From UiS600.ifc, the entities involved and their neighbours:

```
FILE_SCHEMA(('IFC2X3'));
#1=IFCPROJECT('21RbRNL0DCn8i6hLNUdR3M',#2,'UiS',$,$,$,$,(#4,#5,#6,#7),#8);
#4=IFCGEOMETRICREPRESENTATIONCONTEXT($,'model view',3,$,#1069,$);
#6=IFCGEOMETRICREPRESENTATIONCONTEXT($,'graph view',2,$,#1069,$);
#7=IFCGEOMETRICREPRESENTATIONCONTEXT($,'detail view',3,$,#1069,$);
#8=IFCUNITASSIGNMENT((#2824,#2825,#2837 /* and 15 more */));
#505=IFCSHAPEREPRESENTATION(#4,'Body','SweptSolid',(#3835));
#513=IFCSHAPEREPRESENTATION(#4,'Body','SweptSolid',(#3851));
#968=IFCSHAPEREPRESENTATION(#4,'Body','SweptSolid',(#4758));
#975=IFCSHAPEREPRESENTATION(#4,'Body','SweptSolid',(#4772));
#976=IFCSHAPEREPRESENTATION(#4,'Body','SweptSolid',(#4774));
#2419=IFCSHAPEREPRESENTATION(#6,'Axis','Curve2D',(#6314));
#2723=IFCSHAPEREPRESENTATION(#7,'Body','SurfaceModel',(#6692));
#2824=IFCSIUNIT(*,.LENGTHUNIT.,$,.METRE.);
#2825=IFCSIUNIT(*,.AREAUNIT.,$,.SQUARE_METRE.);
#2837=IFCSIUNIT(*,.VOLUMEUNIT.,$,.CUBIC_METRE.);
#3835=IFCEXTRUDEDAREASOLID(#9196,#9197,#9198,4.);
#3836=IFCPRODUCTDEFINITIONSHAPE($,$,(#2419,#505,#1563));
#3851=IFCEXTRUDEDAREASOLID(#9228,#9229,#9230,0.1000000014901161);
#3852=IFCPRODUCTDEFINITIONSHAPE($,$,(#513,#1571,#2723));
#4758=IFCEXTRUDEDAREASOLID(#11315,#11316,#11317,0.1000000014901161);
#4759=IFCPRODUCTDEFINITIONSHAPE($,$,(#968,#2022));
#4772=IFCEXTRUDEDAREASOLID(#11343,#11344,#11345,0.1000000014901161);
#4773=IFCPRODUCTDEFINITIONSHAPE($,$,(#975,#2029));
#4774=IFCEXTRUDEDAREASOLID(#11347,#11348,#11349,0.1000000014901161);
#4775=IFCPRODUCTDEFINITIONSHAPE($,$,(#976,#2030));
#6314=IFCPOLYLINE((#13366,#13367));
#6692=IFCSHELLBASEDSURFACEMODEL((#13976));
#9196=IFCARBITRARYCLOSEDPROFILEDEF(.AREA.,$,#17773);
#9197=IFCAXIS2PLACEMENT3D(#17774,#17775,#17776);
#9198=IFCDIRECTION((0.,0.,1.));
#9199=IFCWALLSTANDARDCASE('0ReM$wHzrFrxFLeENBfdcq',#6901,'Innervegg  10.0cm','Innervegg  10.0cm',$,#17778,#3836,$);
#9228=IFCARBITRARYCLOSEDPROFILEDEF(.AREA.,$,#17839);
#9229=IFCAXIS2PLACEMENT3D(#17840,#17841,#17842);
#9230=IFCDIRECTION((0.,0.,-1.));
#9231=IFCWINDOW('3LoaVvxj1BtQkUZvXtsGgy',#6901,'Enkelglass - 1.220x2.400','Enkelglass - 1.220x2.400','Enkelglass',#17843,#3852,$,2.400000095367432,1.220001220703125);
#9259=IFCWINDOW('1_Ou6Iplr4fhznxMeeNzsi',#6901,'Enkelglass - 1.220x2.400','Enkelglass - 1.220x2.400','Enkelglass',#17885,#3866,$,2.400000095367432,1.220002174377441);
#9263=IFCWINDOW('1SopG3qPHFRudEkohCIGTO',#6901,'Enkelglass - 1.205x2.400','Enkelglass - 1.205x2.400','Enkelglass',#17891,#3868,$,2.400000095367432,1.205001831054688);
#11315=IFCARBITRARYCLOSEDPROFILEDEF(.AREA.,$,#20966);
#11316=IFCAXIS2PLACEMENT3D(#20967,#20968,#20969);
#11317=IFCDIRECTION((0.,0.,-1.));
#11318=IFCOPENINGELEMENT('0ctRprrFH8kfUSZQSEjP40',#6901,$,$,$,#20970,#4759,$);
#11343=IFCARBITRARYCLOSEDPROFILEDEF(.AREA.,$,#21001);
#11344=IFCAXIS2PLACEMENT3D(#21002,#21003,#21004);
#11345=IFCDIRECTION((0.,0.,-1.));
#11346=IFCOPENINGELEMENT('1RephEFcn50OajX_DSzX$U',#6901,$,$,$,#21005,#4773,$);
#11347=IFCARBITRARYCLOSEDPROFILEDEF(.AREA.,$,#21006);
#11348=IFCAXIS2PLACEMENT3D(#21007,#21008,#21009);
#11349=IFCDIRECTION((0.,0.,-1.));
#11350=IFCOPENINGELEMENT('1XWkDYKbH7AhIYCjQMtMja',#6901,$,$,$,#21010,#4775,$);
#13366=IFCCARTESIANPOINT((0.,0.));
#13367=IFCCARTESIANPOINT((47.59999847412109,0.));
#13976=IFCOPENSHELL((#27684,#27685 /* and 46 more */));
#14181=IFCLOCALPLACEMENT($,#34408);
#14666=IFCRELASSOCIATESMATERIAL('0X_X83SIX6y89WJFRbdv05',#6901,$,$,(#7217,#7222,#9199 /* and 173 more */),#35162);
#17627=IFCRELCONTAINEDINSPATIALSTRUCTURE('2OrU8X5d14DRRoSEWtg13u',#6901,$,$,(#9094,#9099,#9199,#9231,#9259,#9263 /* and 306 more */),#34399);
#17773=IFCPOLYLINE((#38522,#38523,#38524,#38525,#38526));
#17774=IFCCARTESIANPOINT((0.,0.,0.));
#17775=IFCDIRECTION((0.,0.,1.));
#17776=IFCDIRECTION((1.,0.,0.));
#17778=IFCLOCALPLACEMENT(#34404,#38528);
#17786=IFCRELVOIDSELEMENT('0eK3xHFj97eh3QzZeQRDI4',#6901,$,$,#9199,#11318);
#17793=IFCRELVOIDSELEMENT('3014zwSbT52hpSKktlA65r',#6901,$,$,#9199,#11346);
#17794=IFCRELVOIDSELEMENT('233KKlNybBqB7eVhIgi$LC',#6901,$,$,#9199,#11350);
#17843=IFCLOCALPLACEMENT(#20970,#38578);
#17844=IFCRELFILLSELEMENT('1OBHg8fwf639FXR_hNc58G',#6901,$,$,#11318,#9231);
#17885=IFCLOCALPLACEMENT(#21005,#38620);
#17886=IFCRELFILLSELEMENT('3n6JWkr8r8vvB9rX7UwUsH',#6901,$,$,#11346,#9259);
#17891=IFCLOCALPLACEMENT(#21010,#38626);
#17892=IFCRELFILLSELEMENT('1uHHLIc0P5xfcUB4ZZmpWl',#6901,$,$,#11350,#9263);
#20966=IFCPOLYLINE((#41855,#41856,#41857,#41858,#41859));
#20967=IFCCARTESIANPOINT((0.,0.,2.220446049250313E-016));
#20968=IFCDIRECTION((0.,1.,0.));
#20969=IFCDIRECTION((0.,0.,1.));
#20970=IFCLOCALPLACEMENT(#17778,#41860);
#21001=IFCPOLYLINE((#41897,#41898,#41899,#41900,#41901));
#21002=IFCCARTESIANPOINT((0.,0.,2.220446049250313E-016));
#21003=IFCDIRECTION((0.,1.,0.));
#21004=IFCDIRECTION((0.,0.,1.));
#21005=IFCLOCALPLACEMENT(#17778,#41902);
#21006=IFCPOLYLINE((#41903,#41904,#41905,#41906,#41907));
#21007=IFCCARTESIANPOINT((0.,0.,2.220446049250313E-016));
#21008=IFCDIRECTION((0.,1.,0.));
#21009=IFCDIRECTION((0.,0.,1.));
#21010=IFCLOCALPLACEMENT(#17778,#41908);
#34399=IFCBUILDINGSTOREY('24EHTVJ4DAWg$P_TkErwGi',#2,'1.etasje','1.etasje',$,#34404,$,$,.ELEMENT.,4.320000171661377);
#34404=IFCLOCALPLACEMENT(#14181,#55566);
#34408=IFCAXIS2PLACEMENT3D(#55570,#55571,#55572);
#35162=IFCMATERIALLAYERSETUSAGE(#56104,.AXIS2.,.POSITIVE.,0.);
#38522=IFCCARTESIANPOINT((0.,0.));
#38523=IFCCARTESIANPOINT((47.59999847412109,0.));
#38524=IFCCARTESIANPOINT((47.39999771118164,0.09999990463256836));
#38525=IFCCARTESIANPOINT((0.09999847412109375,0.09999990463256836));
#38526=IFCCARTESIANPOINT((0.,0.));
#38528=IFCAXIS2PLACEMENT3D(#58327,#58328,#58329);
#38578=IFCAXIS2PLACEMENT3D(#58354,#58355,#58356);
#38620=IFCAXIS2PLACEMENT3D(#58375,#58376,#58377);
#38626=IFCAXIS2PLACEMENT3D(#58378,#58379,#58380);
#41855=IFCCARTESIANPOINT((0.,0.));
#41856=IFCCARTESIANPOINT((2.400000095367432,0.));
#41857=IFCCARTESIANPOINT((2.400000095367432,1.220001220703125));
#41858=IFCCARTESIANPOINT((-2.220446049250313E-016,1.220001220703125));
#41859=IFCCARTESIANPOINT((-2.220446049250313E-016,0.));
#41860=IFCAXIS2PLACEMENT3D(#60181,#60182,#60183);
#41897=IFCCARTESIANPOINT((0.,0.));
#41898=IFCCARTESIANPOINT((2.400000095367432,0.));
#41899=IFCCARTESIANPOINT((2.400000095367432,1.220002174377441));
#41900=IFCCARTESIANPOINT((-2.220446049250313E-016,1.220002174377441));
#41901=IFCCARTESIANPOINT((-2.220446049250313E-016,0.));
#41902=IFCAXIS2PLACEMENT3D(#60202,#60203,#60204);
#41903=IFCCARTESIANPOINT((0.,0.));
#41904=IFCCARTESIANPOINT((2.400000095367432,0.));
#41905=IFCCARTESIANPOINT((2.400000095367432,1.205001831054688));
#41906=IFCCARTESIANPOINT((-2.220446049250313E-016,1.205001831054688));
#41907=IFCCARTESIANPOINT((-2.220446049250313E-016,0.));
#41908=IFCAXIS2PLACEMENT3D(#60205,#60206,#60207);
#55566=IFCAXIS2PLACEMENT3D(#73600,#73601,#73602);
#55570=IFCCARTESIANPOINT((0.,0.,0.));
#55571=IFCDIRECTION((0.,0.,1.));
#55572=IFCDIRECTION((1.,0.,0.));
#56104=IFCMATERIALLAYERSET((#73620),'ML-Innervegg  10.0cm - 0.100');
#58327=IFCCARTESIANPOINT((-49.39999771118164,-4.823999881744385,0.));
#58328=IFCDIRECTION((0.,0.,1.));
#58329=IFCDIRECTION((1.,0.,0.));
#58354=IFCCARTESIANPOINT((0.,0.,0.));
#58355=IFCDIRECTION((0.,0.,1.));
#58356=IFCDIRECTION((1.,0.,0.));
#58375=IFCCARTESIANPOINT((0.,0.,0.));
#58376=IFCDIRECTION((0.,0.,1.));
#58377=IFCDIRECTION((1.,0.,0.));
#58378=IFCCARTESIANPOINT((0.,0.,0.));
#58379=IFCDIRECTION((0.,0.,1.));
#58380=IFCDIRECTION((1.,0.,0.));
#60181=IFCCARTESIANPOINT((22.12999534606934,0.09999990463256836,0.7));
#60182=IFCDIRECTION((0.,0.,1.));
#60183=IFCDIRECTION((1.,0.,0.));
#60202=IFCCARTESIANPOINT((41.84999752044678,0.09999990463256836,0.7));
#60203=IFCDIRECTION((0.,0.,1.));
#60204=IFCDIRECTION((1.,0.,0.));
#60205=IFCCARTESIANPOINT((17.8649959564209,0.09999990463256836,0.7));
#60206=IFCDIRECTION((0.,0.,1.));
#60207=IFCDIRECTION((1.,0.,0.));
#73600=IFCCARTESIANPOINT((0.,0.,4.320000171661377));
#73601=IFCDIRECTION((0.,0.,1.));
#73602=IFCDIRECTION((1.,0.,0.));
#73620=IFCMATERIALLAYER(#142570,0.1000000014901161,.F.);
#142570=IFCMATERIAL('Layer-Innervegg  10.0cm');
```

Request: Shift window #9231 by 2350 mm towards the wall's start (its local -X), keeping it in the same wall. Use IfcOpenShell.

```python
import ifcopenshell
import ifcopenshell.api.geometry
import ifcopenshell.util.placement

model = ifcopenshell.open("UiS600.ifc")

window = model.by_guid("3LoaVvxj1BtQkUZvXtsGgy")
opening = window.FillsVoids[0].RelatingOpeningElement
wall = opening.VoidsElements[0].RelatingBuildingElement

wall_matrix = ifcopenshell.util.placement.get_local_placement(wall.ObjectPlacement)
shift = wall_matrix[:3, 0] * -2.35
before = ifcopenshell.util.placement.get_local_placement(window.ObjectPlacement)[:3, 3].copy()

# The window is placed relative to its opening, so it follows when the opening moves.
matrix = ifcopenshell.util.placement.get_local_placement(opening.ObjectPlacement)
matrix[:3, 3] += shift
ifcopenshell.api.geometry.edit_object_placement(
    model, product=opening, matrix=matrix, is_si=False, should_transform_children=True
)

after = ifcopenshell.util.placement.get_local_placement(window.ObjectPlacement)[:3, 3]
print("window moved by", (after - before).round(3) + 0.0)

model.write("UiS600-out.ifc")
```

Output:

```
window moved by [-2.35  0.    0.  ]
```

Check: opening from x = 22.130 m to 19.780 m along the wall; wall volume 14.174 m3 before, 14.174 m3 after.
